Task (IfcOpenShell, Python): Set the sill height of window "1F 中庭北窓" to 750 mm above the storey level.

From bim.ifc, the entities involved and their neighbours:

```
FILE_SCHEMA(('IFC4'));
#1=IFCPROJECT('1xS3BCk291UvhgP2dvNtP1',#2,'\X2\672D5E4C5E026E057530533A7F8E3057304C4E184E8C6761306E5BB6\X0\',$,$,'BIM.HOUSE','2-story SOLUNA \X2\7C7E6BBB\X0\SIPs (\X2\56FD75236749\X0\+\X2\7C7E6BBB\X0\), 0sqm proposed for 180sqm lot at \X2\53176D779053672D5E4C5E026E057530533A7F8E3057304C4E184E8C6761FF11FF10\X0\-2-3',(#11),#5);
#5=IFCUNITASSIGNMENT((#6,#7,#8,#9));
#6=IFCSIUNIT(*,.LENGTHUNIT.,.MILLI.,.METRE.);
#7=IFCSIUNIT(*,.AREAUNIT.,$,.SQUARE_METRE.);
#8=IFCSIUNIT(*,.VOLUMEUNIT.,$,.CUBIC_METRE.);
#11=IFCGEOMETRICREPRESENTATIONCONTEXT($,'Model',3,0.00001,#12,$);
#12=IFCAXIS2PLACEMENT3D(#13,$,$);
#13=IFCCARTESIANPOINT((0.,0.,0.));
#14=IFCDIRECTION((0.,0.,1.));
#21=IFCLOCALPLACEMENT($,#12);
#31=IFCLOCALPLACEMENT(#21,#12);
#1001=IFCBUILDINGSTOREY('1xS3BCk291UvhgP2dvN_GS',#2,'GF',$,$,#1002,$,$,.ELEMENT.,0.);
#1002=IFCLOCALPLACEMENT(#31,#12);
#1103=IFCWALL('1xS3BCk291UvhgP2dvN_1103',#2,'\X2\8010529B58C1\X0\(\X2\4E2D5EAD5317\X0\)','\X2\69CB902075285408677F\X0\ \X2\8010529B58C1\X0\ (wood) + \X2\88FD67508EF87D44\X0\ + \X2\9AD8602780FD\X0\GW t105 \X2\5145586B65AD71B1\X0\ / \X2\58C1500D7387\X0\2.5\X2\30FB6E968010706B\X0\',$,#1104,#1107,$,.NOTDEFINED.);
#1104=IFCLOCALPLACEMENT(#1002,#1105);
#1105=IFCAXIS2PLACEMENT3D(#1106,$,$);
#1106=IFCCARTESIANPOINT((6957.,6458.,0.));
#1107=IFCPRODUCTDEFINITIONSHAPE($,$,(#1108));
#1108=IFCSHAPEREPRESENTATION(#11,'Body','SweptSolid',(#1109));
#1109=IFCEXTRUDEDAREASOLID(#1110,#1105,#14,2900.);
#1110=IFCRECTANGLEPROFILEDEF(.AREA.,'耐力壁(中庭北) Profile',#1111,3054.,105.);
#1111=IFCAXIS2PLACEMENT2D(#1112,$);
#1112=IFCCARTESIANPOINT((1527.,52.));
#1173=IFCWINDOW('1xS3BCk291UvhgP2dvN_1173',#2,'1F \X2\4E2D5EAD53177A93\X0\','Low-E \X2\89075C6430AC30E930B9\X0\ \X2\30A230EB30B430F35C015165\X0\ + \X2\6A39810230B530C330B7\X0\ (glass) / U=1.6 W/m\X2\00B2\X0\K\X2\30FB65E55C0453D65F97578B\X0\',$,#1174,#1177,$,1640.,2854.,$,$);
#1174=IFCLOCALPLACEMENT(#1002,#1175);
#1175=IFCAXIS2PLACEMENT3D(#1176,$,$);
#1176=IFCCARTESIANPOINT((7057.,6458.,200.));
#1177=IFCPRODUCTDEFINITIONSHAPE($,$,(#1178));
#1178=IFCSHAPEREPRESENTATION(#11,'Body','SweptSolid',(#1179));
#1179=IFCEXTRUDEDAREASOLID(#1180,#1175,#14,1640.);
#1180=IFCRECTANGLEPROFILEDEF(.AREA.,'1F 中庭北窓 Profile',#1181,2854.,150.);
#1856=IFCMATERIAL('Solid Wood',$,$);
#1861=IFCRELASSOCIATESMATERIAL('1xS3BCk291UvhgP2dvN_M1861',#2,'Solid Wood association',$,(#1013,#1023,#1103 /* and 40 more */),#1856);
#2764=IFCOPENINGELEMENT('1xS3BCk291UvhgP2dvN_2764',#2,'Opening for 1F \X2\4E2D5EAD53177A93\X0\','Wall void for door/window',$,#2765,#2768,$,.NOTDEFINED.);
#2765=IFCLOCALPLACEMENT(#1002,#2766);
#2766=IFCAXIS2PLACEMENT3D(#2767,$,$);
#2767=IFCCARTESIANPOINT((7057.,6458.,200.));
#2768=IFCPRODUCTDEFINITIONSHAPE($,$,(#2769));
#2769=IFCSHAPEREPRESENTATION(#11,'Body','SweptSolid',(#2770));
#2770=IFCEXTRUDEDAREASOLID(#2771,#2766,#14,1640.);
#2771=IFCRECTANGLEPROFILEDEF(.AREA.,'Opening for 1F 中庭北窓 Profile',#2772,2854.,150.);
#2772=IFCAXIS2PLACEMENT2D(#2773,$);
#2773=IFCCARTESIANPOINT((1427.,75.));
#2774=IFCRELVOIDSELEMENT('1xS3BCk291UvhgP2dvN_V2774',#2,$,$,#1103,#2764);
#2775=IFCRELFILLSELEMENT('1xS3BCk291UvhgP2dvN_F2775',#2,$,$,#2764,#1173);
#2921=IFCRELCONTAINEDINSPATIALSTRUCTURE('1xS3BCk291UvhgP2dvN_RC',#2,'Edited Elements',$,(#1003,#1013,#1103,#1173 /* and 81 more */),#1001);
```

```python
import numpy as np
import ifcopenshell
import ifcopenshell.api.geometry
import ifcopenshell.geom
import ifcopenshell.util.element
import ifcopenshell.util.placement
import ifcopenshell.util.shape
import ifcopenshell.util.unit

model = ifcopenshell.open("bim.ifc")
unit_scale = ifcopenshell.util.unit.calculate_unit_scale(model)

window = model.by_guid("1xS3BCk291UvhgP2dvN_1173")
opening = window.FillsVoids[0].RelatingOpeningElement
storey = ifcopenshell.util.element.get_container(window, ifc_class="IfcBuildingStorey")
level = ifcopenshell.util.placement.get_local_placement(storey.ObjectPlacement)[2, 3]

# The opening's origin need not be at the sill, so measure its lowest point.
shape = ifcopenshell.geom.create_shape(ifcopenshell.geom.settings(), opening)
bottom = ifcopenshell.util.shape.get_shape_bottom_elevation(shape, shape.geometry) / unit_scale
dz = level + 750.0 - bottom

shift = np.array([0.0, 0.0, dz])
# The window is not placed relative to its opening, so move both.
for product in (opening, window):
    matrix = ifcopenshell.util.placement.get_local_placement(product.ObjectPlacement)
    matrix[:3, 3] += shift
    ifcopenshell.api.geometry.edit_object_placement(model, product=product, matrix=matrix, is_si=False)

print(f"moved by {dz * unit_scale:+.3f} m")

model.write("bim_v2.ifc")
```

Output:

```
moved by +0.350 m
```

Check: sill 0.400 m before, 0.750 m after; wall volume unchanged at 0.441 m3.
